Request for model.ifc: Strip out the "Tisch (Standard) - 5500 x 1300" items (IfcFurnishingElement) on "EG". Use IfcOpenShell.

First a look at what the model holds.

```python
import ifcopenshell
import ifcopenshell.util.element

model = ifcopenshell.open("model.ifc")
print(model.schema)
storey = next(s for s in model.by_type("IfcBuildingStorey") if s.Name == "EG")
furniture = [e for e in ifcopenshell.util.element.get_decomposition(storey) if e.is_a("IfcFurnishingElement")]
seen = {}
for e in furniture:
    element_type = ifcopenshell.util.element.get_type(e)
    name = element_type.Name if element_type not in (None, e) else None
    seen[name] = seen.get(name, 0) + 1
for name, count in sorted(seen.items(), key=str):
    print(count, "x", name)
```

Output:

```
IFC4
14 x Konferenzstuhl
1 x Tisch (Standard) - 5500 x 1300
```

```python
import ifcopenshell
import ifcopenshell.api.root
import ifcopenshell.util.element

model = ifcopenshell.open("model.ifc")

storey = next(s for s in model.by_type("IfcBuildingStorey") if s.Name == "EG")
furniture = [e for e in ifcopenshell.util.element.get_decomposition(storey) if e.is_a("IfcFurnishingElement")]
targets = [e for e in furniture if (t := ifcopenshell.util.element.get_type(e)) not in (None, e) and t.Name == "Tisch (Standard) - 5500 x 1300"]

for e in targets:
    ifcopenshell.api.root.remove_product(model, product=e)
print(len(targets), "removed")

model.write("model_edited.ifc")
```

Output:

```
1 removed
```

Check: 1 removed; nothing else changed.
